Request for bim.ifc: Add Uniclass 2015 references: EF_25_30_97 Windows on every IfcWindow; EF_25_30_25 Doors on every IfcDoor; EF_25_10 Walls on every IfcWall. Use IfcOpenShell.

First a look at what the model holds.

```python
import ifcopenshell

model = ifcopenshell.open("bim.ifc")
print(model.schema)
print("classifications:", [c.Name for c in model.by_type("IfcClassification")])
for ifc_class in ("IfcDoor", "IfcRoof", "IfcStair", "IfcWall", "IfcWindow"):
    print(ifc_class, len(model.by_type(ifc_class)))
```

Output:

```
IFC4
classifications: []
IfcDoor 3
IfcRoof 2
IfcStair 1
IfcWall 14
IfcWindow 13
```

```python
import ifcopenshell
import ifcopenshell.api.classification

model = ifcopenshell.open("bim.ifc")

system = ifcopenshell.api.classification.add_classification(model, classification="Uniclass 2015")

codes = {
    "IfcWindow": ("EF_25_30_97", "Windows"),
    "IfcDoor": ("EF_25_30_25", "Doors"),
    "IfcWall": ("EF_25_10", "Walls"),
}
for ifc_class, (code, name) in codes.items():
    products = model.by_type(ifc_class)
    ifcopenshell.api.classification.add_reference(
        model, products=products, classification=system, identification=code, name=name
    )
    print(code, len(products))

model.write("bim_updated.ifc")
```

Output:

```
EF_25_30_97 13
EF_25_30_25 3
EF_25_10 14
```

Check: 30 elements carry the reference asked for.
